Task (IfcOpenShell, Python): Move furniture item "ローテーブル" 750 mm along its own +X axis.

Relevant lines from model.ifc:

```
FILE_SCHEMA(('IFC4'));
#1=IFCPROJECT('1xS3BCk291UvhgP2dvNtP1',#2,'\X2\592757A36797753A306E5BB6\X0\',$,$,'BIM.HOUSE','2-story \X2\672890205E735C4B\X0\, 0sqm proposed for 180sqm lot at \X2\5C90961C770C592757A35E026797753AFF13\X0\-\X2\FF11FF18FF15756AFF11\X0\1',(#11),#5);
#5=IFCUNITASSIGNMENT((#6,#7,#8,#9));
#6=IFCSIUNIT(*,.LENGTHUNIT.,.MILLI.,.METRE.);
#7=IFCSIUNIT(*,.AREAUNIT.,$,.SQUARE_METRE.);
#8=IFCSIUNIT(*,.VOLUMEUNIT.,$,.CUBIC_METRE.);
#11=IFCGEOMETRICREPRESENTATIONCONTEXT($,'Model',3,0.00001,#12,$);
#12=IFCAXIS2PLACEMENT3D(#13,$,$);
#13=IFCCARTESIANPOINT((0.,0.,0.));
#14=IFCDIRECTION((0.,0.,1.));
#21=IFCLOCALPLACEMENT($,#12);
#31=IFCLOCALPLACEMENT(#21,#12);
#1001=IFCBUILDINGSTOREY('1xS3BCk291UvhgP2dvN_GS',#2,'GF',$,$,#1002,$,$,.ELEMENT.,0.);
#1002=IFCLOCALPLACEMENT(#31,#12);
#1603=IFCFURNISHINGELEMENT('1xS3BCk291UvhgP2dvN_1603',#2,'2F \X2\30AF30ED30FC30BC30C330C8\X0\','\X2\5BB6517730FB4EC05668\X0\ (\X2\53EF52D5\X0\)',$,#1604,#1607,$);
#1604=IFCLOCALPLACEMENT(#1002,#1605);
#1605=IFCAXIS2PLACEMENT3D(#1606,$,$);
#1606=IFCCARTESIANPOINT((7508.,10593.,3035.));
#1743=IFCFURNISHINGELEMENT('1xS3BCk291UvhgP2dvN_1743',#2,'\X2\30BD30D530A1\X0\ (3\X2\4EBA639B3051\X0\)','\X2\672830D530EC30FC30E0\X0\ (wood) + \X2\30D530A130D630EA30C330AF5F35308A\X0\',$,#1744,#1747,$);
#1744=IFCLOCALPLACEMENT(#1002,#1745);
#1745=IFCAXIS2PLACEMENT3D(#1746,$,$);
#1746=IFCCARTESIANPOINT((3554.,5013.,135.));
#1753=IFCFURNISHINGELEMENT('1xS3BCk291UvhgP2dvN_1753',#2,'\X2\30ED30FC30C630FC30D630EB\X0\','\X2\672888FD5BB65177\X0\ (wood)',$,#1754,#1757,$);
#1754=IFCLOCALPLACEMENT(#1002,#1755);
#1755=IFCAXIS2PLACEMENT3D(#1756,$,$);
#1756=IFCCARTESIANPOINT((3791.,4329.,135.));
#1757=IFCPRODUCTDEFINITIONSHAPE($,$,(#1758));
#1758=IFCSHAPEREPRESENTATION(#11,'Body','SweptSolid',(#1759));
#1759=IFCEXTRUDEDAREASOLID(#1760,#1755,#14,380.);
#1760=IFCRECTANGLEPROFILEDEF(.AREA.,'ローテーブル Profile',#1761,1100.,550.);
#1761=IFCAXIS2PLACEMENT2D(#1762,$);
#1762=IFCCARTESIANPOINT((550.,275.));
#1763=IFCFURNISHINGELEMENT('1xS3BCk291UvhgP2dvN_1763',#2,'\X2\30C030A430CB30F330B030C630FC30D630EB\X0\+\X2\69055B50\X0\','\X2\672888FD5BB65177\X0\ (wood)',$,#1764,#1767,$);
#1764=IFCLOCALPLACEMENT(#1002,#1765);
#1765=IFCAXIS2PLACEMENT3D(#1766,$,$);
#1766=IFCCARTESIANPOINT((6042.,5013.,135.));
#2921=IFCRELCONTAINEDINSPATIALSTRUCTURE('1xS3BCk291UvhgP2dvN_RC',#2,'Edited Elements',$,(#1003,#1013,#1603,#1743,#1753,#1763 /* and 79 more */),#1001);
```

```python
import ifcopenshell
import ifcopenshell.api.geometry
import ifcopenshell.util.placement
import ifcopenshell.util.unit

model = ifcopenshell.open("model.ifc")
unit_scale = ifcopenshell.util.unit.calculate_unit_scale(model)

item = model.by_guid("1xS3BCk291UvhgP2dvN_1753")
matrix = ifcopenshell.util.placement.get_local_placement(item.ObjectPlacement)
matrix[:3, 3] += matrix[:3, 0] * 0.75 / unit_scale
ifcopenshell.api.geometry.edit_object_placement(model, product=item, matrix=matrix, is_si=False)

print(ifcopenshell.util.placement.get_local_placement(item.ObjectPlacement).round(3) + 0.0)

model.write("model_updated.ifc")
```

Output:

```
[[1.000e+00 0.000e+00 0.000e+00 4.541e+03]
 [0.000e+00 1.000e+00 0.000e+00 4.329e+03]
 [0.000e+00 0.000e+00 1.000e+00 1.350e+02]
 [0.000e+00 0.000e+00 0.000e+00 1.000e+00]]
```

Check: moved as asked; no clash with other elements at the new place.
